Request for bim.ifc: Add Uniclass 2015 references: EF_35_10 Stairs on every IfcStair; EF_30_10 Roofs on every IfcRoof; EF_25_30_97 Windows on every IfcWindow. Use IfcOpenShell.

First a look at what the model holds.

```python
import ifcopenshell

model = ifcopenshell.open("bim.ifc")
print(model.schema)
print("classifications:", [c.Name for c in model.by_type("IfcClassification")])
for ifc_class in ("IfcDoor", "IfcRoof", "IfcStair", "IfcWall", "IfcWindow"):
    print(ifc_class, len(model.by_type(ifc_class)))
```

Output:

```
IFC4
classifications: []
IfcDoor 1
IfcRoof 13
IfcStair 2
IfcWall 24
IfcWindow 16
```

```python
import ifcopenshell
import ifcopenshell.api.classification

model = ifcopenshell.open("bim.ifc")

system = ifcopenshell.api.classification.add_classification(model, classification="Uniclass 2015")

codes = {
    "IfcStair": ("EF_35_10", "Stairs"),
    "IfcRoof": ("EF_30_10", "Roofs"),
    "IfcWindow": ("EF_25_30_97", "Windows"),
}
for ifc_class, (code, name) in codes.items():
    products = model.by_type(ifc_class)
    ifcopenshell.api.classification.add_reference(
        model, products=products, classification=system, identification=code, name=name
    )
    print(code, len(products))

model.write("bim_v2.ifc")
```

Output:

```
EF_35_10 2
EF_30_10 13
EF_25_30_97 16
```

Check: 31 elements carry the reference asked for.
